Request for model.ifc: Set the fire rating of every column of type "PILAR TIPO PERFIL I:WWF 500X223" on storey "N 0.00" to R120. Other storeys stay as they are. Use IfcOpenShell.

First a look at what the model holds.

```python
import ifcopenshell
import ifcopenshell.util.element

model = ifcopenshell.open("model.ifc")
print(model.schema)
storey = next(s for s in model.by_type("IfcBuildingStorey") if s.Name == "N 0.00")
columns = [e for e in ifcopenshell.util.element.get_decomposition(storey) if e.is_a("IfcColumn")]
seen = {}
for e in columns:
    element_type = ifcopenshell.util.element.get_type(e)
    key = (element_type.Name if element_type != e and element_type else None, ifcopenshell.util.element.get_pset(e, "Pset_ColumnCommon", "FireRating"))
    seen[key] = seen.get(key, 0) + 1
for (name, value), count in sorted(seen.items(), key=str):
    print(count, "x", name, "|", value)
```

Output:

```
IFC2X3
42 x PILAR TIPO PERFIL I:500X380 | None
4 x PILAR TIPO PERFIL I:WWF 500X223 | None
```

```python
import ifcopenshell
import ifcopenshell.api.pset
import ifcopenshell.util.element

model = ifcopenshell.open("model.ifc")

storey = next(s for s in model.by_type("IfcBuildingStorey") if s.Name == "N 0.00")
columns = [e for e in ifcopenshell.util.element.get_decomposition(storey) if e.is_a("IfcColumn")]

count = 0
for e in columns:
    element_type = ifcopenshell.util.element.get_type(e)
    if element_type in (None, e) or element_type.Name != "PILAR TIPO PERFIL I:WWF 500X223":
        continue
    # add_pset returns the element's existing set when there is one.
    pset = ifcopenshell.api.pset.add_pset(model, product=e, name="Pset_ColumnCommon")
    ifcopenshell.api.pset.edit_pset(model, pset=pset, properties={"FireRating": "R120"})
    count += 1

print(count, "columns updated")

model.write("model_edited.ifc")
```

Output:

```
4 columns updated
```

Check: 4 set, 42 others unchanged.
